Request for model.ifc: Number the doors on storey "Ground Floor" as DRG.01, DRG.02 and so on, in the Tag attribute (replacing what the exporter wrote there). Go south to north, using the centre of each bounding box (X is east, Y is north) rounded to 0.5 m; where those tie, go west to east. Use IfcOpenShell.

First a look at what the model holds.

```python
import ifcopenshell
import ifcopenshell.util.element
import ifcopenshell.util.placement

model = ifcopenshell.open("model.ifc")
print(model.schema)
storey = next(s for s in model.by_type("IfcBuildingStorey") if s.Name == "Ground Floor")
doors = [e for e in ifcopenshell.util.element.get_decomposition(storey) if e.is_a("IfcDoor")]
for e in sorted(doors, key=lambda e: e.id()):
    origin = ifcopenshell.util.placement.get_local_placement(e.ObjectPlacement)[:3, 3]
    print(e.id(), e.Tag, e.Name, origin.round(2) + 0.0, sep=" | ")
```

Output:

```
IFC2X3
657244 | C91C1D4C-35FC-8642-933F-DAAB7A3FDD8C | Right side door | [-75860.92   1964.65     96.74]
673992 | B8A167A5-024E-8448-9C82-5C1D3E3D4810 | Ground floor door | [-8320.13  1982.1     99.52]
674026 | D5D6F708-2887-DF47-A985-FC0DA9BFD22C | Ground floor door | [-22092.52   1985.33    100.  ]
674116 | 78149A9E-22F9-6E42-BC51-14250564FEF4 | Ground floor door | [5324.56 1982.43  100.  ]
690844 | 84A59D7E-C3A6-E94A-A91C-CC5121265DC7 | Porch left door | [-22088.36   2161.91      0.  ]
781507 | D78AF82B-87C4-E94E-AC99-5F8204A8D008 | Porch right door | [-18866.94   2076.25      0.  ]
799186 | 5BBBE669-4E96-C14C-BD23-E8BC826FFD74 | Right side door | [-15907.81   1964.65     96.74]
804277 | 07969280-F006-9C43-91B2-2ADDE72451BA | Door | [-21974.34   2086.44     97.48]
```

```python
import ifcopenshell
import ifcopenshell.geom
import ifcopenshell.util.element
import ifcopenshell.util.shape

model = ifcopenshell.open("model.ifc")
settings = ifcopenshell.geom.settings()
settings.set("use-world-coords", True)


def centre(element):
    shape = ifcopenshell.geom.create_shape(settings, element)
    return ifcopenshell.util.shape.get_bbox_centroid(shape.geometry)


storey = next(s for s in model.by_type("IfcBuildingStorey") if s.Name == "Ground Floor")
doors = [e for e in ifcopenshell.util.element.get_decomposition(storey) if e.is_a("IfcDoor")]

# Insertion points can sit at a corner or the storey origin, so sort by the geometry (in metres).
centres = {e: centre(e) for e in doors}
doors.sort(key=lambda e: (round(centres[e][1] / 0.5), centres[e][0]))

for i, e in enumerate(doors, start=1):
    number = f"DRG.{i:02d}"
    e.Tag = number
    print(e.id(), number)

model.write("model-out.ifc")
```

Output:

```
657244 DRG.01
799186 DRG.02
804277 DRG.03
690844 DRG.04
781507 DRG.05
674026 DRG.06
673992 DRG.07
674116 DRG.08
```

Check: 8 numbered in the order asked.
